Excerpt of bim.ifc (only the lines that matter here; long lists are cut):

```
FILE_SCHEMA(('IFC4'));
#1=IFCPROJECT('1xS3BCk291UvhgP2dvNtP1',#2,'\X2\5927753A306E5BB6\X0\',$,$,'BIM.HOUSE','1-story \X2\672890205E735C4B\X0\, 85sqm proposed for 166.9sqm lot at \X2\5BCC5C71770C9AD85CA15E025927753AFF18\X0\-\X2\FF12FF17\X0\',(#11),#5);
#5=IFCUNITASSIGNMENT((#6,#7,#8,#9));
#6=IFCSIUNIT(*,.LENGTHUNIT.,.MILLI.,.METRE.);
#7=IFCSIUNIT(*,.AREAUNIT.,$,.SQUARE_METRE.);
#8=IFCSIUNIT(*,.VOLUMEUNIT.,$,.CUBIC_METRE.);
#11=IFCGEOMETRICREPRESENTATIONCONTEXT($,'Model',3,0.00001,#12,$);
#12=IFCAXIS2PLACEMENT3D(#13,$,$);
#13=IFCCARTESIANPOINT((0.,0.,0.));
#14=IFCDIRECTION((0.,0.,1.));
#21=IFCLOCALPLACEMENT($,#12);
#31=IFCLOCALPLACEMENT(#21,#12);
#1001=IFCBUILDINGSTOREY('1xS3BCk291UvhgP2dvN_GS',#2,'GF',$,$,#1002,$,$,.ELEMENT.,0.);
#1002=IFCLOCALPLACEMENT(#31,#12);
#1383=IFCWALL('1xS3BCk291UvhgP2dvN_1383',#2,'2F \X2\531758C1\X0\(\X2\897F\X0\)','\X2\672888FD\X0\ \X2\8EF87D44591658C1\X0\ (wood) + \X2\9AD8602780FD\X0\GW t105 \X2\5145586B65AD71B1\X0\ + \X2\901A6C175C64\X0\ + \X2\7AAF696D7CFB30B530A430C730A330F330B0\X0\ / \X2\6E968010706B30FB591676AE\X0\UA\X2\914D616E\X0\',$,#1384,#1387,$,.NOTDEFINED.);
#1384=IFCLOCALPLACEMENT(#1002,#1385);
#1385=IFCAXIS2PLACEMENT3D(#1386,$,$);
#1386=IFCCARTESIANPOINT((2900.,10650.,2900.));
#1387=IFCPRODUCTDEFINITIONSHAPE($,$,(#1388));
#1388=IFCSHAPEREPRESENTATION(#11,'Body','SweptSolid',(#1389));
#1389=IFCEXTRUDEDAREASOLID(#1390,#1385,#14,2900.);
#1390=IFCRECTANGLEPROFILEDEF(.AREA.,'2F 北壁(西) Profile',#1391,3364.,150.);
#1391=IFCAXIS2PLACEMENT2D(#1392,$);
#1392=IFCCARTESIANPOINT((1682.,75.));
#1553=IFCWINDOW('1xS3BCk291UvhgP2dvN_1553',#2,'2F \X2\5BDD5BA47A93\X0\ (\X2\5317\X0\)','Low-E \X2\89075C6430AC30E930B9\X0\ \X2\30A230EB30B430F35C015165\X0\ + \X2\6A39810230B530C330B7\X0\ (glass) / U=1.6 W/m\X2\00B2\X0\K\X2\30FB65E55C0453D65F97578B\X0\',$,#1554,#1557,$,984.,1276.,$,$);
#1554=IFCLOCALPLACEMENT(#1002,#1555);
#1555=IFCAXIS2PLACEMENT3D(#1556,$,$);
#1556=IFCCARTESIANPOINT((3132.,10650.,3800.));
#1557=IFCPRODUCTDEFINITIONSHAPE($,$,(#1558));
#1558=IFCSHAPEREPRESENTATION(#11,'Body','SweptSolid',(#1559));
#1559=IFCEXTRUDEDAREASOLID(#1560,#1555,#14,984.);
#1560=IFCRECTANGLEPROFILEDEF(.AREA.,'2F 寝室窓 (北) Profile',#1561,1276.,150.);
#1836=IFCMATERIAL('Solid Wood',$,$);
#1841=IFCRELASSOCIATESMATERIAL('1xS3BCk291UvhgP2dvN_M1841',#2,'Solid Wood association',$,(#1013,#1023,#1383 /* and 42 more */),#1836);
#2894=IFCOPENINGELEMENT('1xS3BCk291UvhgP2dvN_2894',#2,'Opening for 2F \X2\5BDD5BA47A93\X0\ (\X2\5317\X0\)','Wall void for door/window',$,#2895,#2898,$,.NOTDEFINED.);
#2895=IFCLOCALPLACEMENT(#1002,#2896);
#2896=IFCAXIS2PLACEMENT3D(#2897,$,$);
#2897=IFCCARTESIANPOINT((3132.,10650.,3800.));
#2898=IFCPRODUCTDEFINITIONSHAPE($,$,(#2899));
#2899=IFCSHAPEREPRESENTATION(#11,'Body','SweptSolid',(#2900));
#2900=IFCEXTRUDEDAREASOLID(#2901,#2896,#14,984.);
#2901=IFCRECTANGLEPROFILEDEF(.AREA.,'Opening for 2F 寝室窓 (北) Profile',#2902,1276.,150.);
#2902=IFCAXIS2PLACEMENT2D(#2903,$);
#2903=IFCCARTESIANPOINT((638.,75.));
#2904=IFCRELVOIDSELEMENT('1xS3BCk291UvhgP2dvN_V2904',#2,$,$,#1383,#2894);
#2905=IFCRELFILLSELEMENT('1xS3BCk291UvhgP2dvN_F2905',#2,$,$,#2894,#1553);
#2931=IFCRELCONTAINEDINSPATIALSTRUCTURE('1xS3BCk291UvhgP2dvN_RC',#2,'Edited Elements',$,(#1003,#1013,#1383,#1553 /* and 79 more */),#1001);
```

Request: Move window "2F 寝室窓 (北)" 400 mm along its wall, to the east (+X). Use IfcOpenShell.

```python
import ifcopenshell
import ifcopenshell.api.geometry
import ifcopenshell.util.placement

model = ifcopenshell.open("bim.ifc")

window = model.by_guid("1xS3BCk291UvhgP2dvN_1553")
opening = window.FillsVoids[0].RelatingOpeningElement
wall = opening.VoidsElements[0].RelatingBuildingElement

wall_matrix = ifcopenshell.util.placement.get_local_placement(wall.ObjectPlacement)
shift = wall_matrix[:3, 0] * 400.0
before = ifcopenshell.util.placement.get_local_placement(window.ObjectPlacement)[:3, 3].copy()

# The window is not placed relative to its opening, so move both.
for product in (opening, window):
    matrix = ifcopenshell.util.placement.get_local_placement(product.ObjectPlacement)
    matrix[:3, 3] += shift
    ifcopenshell.api.geometry.edit_object_placement(model, product=product, matrix=matrix, is_si=False)

after = ifcopenshell.util.placement.get_local_placement(window.ObjectPlacement)[:3, 3]
print("window moved by", (after - before).round(3) + 0.0)

model.write("bim_updated.ifc")
```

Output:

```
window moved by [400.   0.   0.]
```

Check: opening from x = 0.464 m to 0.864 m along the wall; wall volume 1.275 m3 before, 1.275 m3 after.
